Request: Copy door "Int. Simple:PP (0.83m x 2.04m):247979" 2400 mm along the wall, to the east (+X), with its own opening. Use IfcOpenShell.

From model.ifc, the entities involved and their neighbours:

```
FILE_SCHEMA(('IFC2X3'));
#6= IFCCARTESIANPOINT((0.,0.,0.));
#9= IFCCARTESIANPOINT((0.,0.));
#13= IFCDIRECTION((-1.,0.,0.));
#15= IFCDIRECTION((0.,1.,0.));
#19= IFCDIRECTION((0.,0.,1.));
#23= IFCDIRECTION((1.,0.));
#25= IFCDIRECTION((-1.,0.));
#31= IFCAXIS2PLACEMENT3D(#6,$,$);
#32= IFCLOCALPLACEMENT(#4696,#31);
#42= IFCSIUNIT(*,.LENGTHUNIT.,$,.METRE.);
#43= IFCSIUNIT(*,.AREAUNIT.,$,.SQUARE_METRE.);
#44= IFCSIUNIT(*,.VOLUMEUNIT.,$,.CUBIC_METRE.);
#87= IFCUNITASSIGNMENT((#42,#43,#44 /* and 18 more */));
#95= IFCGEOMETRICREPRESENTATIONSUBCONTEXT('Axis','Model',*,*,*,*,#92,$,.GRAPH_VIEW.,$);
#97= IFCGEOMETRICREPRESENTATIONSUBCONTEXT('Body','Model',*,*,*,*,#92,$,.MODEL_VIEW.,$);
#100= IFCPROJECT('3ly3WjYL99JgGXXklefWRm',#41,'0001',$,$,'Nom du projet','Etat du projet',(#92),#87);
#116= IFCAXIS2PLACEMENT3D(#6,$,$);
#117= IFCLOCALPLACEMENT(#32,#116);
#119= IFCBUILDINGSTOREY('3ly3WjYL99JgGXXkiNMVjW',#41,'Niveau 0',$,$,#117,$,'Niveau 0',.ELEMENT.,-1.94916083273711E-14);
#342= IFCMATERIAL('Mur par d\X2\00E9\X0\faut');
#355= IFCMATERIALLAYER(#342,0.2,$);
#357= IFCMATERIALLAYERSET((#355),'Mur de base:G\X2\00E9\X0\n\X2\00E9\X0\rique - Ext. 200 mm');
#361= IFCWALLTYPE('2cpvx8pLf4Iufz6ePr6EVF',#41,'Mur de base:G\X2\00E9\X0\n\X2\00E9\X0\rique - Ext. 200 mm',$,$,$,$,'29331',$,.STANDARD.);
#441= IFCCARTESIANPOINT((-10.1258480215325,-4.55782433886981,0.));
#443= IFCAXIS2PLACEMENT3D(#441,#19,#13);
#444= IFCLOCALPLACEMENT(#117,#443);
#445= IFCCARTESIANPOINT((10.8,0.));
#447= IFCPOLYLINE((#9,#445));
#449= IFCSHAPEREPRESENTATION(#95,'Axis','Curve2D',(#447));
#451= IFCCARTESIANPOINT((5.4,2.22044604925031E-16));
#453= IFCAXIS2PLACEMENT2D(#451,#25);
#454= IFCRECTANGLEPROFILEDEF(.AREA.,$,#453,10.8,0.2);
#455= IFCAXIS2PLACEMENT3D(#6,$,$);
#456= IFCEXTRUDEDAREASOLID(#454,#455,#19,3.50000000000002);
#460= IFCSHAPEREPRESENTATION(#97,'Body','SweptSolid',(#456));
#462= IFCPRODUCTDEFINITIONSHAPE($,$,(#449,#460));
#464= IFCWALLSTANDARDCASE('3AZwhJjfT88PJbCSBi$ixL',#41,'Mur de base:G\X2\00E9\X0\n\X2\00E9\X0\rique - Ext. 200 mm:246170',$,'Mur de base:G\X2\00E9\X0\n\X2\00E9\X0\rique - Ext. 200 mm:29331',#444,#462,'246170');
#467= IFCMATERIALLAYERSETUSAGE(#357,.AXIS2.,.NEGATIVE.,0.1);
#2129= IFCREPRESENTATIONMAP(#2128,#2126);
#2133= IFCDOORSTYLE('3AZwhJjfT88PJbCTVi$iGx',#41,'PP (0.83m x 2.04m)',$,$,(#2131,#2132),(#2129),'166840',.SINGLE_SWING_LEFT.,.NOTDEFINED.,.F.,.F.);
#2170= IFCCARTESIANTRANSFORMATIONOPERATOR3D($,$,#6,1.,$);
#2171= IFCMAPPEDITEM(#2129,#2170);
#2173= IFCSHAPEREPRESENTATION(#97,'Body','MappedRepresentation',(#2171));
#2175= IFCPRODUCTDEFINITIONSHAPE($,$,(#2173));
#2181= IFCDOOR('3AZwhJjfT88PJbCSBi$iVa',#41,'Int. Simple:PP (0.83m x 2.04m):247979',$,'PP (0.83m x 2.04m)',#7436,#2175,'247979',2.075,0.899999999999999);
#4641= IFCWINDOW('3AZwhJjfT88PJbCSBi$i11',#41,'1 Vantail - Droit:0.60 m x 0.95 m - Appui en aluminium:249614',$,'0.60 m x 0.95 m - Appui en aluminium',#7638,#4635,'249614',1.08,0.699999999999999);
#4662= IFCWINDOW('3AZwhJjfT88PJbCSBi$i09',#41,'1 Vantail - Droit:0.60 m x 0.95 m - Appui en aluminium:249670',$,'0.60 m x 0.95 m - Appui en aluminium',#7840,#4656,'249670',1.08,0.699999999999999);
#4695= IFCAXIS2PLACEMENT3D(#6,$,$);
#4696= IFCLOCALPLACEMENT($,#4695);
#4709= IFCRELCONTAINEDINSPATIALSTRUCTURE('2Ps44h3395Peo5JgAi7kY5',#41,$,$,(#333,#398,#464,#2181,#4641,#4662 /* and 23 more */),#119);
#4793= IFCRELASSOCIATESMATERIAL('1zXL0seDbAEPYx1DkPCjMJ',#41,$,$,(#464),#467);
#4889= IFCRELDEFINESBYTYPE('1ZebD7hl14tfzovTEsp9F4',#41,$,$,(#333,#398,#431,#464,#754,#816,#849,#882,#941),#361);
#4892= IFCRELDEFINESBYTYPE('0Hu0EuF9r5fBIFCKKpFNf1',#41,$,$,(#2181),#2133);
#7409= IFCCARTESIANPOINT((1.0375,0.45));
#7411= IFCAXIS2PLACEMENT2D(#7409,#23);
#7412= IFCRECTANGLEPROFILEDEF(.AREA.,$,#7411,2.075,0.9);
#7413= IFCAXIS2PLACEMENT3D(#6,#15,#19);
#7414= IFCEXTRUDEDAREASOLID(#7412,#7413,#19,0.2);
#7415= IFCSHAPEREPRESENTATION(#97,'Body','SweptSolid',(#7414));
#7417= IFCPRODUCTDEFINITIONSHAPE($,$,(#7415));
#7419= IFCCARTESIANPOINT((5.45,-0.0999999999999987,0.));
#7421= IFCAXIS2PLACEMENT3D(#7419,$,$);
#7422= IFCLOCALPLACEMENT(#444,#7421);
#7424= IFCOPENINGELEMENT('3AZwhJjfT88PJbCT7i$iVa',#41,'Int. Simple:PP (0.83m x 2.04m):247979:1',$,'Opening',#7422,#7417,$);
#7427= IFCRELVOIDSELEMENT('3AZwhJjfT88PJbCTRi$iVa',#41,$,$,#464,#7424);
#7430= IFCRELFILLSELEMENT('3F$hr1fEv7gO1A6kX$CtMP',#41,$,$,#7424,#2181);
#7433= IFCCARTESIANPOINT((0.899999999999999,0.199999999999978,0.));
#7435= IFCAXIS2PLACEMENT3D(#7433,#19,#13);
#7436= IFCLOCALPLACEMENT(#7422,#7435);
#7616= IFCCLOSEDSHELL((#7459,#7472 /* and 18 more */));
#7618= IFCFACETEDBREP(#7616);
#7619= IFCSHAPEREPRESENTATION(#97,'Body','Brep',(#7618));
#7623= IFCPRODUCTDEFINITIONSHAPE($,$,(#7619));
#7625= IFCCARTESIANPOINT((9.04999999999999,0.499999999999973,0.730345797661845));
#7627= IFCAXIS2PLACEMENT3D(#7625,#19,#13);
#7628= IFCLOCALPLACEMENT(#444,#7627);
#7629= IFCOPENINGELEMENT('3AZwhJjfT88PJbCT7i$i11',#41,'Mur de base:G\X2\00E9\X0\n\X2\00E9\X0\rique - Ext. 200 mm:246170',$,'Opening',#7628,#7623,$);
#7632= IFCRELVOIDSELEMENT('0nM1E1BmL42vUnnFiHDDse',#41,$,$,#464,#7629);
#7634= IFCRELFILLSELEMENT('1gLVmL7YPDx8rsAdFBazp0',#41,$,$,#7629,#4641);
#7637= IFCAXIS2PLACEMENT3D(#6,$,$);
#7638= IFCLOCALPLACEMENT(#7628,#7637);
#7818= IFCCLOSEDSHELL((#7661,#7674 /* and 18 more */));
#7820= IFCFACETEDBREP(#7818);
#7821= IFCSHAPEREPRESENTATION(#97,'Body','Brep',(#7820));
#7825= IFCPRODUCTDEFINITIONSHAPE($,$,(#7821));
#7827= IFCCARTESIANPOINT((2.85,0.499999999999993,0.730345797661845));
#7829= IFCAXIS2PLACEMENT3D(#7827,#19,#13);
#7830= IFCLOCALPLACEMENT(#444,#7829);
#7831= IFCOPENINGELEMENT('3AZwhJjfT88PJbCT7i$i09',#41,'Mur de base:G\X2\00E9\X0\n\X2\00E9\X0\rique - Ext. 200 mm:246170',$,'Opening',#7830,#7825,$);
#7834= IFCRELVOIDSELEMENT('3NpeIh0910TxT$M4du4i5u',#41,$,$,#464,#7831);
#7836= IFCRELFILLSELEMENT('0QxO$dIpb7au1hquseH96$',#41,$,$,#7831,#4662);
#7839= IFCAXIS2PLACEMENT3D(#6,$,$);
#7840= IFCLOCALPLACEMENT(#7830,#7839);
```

```python
import ifcopenshell
import ifcopenshell.api.feature
import ifcopenshell.api.geometry
import ifcopenshell.api.root
import ifcopenshell.geom
import ifcopenshell.util.element
import ifcopenshell.util.placement
import ifcopenshell.util.shape
import ifcopenshell.util.unit

model = ifcopenshell.open("model.ifc")
unit_scale = ifcopenshell.util.unit.calculate_unit_scale(model)
settings = ifcopenshell.geom.settings()


def volume(element):
    """Net volume in cubic metres, openings subtracted."""
    shape = ifcopenshell.geom.create_shape(settings, element)
    return ifcopenshell.util.shape.get_volume(shape.geometry)


def reuse_history(source, copy):
    """copy_class also copies each property set's owner history, people and application; keep the originals."""
    for rel in copy.IsDefinedBy:
        if rel.is_a("IfcRelDefinesByProperties") and (history := rel.RelatingPropertyDefinition.OwnerHistory):
            rel.RelatingPropertyDefinition.OwnerHistory = source.OwnerHistory
            ifcopenshell.util.element.remove_deep2(model, history)


door = model.by_id(2181)
opening = door.FillsVoids[0].RelatingOpeningElement
wall = opening.VoidsElements[0].RelatingBuildingElement
before = volume(wall)
shift = ifcopenshell.util.placement.get_local_placement(wall.ObjectPlacement)[:3, 0] * -2.4 / unit_scale

# copy_class copies the void relationship, type, container and properties, but no geometry.
new_opening = ifcopenshell.api.root.copy_class(model, product=opening)
new_opening.Representation = ifcopenshell.util.element.copy_deep(
    model, opening.Representation, exclude=["IfcGeometricRepresentationContext", "IfcRepresentationMap"]
)
new_opening.Name = "Int. Simple:PP (0.83m x 2.04m)"
new_door = ifcopenshell.api.root.copy_class(model, product=door)
new_door.Representation = ifcopenshell.util.element.copy_deep(
    model, door.Representation, exclude=["IfcGeometricRepresentationContext", "IfcRepresentationMap"]
)
new_door.Name = "Int. Simple:PP (0.83m x 2.04m)"
new_door.Tag = None
reuse_history(door, new_door)
fills = ifcopenshell.api.feature.add_filling(model, opening=new_opening, element=new_door)
fills.OwnerHistory = new_door.OwnerHistory  # required in IFC2X3

for old, new in ((opening, new_opening), (door, new_door)):
    matrix = ifcopenshell.util.placement.get_local_placement(old.ObjectPlacement)
    matrix[:3, 3] += shift
    ifcopenshell.api.geometry.edit_object_placement(model, product=new, matrix=matrix, is_si=False)

after = volume(wall)

print(f"wall volume {before:.3f} -> {after:.3f} m3")

model.write("model_edited.ifc")
```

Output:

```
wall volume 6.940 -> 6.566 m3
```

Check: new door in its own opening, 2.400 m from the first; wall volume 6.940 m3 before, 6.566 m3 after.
